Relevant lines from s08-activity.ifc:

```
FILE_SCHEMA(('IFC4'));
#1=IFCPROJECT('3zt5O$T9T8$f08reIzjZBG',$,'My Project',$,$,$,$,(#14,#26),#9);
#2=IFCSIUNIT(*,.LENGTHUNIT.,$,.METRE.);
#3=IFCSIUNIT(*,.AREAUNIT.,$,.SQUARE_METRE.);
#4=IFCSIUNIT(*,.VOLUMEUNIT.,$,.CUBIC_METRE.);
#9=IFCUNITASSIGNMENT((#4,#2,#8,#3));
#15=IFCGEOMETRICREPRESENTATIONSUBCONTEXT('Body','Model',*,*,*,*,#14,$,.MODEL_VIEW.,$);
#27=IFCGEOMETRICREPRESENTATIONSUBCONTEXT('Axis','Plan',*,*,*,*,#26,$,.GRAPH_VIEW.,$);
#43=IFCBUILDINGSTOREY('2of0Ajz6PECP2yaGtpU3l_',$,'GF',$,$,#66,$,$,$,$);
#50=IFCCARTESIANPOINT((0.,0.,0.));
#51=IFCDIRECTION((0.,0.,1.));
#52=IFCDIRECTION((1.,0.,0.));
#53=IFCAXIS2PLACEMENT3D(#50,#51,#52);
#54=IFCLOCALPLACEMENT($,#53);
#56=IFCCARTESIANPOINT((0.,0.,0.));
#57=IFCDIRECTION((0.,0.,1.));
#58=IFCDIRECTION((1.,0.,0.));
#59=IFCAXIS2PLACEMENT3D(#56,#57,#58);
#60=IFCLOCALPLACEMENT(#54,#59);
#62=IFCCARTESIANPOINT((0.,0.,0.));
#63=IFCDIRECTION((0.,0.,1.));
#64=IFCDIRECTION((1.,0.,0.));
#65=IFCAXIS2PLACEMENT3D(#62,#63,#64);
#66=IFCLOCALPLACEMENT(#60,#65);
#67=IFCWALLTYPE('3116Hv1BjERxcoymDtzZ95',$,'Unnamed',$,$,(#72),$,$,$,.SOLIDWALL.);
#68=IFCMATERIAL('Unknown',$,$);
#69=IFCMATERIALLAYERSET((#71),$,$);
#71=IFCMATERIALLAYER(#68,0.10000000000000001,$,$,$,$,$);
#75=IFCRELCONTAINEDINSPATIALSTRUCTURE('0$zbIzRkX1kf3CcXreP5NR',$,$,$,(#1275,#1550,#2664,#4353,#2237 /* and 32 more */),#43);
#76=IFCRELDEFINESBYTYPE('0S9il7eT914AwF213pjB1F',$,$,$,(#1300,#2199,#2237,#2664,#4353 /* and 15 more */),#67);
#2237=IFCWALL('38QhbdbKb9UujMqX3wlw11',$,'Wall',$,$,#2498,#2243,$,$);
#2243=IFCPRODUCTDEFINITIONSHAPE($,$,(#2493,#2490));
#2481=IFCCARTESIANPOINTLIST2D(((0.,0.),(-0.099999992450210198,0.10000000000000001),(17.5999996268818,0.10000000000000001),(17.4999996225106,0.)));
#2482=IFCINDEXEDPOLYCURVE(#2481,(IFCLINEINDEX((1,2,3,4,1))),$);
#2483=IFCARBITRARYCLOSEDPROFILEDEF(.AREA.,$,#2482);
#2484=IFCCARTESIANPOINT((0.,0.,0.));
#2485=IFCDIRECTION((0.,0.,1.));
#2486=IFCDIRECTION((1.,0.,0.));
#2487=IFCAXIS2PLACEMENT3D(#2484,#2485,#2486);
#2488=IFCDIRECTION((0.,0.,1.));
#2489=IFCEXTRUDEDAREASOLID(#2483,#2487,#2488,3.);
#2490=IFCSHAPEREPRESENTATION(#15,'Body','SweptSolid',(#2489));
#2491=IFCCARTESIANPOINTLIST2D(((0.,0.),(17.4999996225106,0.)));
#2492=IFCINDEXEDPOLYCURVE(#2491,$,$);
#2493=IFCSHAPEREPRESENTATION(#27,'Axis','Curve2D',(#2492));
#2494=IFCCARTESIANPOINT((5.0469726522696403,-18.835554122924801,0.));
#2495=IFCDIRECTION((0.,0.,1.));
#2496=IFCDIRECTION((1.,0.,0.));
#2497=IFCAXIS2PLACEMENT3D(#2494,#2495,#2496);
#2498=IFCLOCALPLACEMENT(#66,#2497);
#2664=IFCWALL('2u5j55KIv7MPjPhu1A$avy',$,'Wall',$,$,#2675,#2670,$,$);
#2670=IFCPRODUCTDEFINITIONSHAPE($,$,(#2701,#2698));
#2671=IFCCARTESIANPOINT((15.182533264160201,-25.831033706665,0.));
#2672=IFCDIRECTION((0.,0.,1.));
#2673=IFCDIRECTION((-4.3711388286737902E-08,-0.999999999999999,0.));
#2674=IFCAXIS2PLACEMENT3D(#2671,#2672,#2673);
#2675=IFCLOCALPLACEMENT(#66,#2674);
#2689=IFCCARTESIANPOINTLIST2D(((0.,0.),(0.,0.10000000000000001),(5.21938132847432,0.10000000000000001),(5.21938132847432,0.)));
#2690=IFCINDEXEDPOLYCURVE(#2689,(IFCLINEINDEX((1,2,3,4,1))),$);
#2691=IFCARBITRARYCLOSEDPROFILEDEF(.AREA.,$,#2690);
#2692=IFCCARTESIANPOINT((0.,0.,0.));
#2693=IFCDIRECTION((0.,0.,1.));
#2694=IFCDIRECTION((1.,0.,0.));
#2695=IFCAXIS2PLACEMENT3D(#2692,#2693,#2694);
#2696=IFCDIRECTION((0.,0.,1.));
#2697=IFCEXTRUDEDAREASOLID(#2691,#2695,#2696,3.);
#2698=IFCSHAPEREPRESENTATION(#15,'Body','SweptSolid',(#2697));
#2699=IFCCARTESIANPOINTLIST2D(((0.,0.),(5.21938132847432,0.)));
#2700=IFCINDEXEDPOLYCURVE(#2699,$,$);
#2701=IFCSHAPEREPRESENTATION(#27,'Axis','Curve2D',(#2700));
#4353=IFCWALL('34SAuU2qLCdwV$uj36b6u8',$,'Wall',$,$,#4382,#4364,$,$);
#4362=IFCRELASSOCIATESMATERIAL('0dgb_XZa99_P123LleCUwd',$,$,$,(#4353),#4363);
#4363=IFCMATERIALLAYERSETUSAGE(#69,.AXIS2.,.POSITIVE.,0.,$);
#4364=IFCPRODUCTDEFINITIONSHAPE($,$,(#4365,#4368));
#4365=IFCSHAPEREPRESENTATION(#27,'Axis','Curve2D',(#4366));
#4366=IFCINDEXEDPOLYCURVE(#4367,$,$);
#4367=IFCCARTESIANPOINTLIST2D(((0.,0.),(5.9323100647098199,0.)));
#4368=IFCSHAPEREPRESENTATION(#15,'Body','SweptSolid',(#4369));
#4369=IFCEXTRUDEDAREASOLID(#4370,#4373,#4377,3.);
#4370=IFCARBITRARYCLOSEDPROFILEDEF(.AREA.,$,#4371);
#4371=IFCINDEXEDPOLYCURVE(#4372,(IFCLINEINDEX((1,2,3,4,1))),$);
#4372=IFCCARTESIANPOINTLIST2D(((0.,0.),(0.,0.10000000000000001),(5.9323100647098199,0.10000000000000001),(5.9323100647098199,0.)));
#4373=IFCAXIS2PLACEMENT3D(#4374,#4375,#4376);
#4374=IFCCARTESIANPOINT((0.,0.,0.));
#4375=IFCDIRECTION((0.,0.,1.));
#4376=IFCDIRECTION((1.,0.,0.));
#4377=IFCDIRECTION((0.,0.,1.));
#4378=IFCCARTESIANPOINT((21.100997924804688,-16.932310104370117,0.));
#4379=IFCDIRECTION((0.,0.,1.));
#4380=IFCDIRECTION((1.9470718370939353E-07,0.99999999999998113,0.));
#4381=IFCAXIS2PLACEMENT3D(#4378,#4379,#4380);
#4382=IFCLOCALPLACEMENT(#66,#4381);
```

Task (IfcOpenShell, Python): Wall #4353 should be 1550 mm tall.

```python
import ifcopenshell
import ifcopenshell.geom
import ifcopenshell.util.representation
import ifcopenshell.util.shape

model = ifcopenshell.open("s08-activity.ifc")
settings = ifcopenshell.geom.settings()


def volume(element):
    """Net volume in cubic metres, openings subtracted."""
    shape = ifcopenshell.geom.create_shape(settings, element)
    return ifcopenshell.util.shape.get_volume(shape.geometry)


wall = model.by_guid("34SAuU2qLCdwV$uj36b6u8")
before = volume(wall)

body = ifcopenshell.util.representation.get_representation(wall, "Model", "Body")
solid = body.Items[0]
old_height = solid.Depth
solid.Depth = 1.55
after = volume(wall)

print(f"height {old_height:g} -> {solid.Depth:g}, volume {before:.3f} -> {after:.3f} m3")

model.write("s08-activity_v2.ifc")
```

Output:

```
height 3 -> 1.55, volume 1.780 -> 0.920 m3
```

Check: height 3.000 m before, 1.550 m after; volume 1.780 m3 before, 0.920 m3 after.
